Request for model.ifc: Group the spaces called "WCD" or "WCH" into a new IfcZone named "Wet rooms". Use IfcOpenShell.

First a look at what the model holds.

```python
import ifcopenshell

model = ifcopenshell.open("model.ifc")
print(model.schema)
seen = {}
for space in model.by_type("IfcSpace"):
    seen[space.LongName] = seen.get(space.LongName, 0) + 1
for name, count in sorted(seen.items(), key=str):
    print(count, "x", name)
print("zones:", [z.Name for z in model.by_type("IfcZone")][:20])
```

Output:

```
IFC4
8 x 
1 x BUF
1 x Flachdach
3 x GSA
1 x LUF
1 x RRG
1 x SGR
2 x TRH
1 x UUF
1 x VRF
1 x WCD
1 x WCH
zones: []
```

```python
import ifcopenshell
import ifcopenshell.api.group
import ifcopenshell.api.root

model = ifcopenshell.open("model.ifc")

names = {"WCD", "WCH"}
spaces = [s for s in model.by_type("IfcSpace") if s.LongName in names]

zone = ifcopenshell.api.root.create_entity(model, ifc_class="IfcZone", name="Wet rooms")
ifcopenshell.api.group.assign_group(model, products=spaces, group=zone)
print(len(spaces), "spaces in", zone.Name)

model.write("model_edited.ifc")
```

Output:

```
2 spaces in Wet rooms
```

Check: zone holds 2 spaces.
